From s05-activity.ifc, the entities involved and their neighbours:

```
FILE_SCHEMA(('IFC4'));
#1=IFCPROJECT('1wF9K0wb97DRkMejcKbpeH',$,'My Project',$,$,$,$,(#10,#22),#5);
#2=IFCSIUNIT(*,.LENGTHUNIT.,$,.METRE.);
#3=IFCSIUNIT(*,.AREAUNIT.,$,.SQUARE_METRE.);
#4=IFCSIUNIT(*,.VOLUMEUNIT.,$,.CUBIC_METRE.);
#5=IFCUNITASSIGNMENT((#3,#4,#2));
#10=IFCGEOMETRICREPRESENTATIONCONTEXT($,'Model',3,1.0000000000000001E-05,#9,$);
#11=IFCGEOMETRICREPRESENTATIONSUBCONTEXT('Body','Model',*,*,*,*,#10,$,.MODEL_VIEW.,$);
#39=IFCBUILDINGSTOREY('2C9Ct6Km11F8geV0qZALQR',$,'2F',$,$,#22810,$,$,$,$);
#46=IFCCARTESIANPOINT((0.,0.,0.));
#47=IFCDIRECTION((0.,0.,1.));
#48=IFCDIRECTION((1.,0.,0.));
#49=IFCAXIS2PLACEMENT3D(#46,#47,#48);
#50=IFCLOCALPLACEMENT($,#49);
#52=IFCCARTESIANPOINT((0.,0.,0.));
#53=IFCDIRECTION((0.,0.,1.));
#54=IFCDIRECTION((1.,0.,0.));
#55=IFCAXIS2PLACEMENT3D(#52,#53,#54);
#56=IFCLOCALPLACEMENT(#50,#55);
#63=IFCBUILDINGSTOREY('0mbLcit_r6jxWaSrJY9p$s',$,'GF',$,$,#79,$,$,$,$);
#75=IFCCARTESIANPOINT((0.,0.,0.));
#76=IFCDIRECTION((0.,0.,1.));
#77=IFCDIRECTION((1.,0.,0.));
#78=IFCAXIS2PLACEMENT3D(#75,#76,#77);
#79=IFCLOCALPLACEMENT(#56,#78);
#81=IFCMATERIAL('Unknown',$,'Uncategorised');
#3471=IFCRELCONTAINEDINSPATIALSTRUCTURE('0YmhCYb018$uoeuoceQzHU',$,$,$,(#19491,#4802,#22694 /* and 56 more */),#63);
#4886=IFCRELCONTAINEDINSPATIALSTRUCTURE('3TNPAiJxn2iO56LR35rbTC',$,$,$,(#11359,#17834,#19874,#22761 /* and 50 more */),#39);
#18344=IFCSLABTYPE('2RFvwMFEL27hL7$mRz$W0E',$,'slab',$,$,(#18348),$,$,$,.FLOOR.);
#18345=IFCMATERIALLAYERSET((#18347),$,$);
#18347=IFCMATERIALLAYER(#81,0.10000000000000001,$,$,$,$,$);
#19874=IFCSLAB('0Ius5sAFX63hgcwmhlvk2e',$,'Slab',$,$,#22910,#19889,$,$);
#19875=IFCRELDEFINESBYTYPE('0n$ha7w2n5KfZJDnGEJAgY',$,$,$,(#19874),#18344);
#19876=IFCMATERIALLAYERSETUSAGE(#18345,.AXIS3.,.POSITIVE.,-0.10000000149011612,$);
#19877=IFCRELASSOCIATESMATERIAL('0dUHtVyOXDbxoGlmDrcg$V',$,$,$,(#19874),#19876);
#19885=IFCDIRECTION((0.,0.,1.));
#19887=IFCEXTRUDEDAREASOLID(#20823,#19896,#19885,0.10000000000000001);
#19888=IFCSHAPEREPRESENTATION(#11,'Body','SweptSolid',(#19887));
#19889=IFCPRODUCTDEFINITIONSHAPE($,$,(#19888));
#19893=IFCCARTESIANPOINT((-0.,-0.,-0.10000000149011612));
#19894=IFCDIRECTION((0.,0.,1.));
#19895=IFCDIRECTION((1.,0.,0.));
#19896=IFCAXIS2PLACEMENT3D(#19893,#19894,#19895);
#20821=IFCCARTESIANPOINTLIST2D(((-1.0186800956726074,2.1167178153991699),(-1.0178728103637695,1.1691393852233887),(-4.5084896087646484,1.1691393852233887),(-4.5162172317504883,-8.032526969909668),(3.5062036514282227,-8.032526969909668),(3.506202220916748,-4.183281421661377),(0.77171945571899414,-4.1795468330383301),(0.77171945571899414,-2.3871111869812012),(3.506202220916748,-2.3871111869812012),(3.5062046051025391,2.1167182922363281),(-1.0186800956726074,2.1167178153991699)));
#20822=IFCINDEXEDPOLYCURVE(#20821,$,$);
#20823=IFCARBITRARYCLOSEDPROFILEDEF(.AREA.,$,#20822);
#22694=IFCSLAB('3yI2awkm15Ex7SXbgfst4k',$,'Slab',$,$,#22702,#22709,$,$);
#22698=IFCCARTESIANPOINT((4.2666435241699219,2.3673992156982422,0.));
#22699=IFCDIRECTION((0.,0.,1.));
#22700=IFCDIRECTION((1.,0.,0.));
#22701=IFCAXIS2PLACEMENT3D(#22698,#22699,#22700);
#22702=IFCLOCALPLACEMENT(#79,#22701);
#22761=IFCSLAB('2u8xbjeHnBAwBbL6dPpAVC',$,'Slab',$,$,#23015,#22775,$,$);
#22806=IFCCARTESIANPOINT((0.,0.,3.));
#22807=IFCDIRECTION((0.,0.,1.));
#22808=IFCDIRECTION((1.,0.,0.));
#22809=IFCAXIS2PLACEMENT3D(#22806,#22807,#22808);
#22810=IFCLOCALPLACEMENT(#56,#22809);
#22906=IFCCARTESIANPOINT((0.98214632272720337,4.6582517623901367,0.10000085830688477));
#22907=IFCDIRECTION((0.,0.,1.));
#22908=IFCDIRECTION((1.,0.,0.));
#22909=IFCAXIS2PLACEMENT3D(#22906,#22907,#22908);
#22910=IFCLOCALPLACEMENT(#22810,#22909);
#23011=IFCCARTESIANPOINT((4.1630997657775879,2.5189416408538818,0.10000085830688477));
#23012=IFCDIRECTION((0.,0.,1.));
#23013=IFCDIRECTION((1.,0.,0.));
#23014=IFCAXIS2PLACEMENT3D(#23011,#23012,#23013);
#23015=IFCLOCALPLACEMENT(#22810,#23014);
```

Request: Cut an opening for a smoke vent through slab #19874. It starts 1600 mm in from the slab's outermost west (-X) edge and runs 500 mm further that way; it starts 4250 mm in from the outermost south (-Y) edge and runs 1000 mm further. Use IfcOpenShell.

```python
import numpy as np
import ifcopenshell
import ifcopenshell.api.feature
import ifcopenshell.api.geometry
import ifcopenshell.api.root
import ifcopenshell.geom
import ifcopenshell.util.placement
import ifcopenshell.util.representation
import ifcopenshell.util.shape
import ifcopenshell.util.unit

model = ifcopenshell.open("s05-activity.ifc")
unit_scale = ifcopenshell.util.unit.calculate_unit_scale(model)
settings = ifcopenshell.geom.settings()


def volume(element):
    """Net volume in cubic metres, openings subtracted."""
    shape = ifcopenshell.geom.create_shape(settings, element)
    return ifcopenshell.util.shape.get_volume(shape.geometry)


slab = model.by_guid("0Ius5sAFX63hgcwmhlvk2e")
before = volume(slab)

# Extent in the slab's own axes, in metres. The edges named are its -X and -Y sides.
slab_shape = ifcopenshell.geom.create_shape(settings, slab)
vertices = ifcopenshell.util.shape.get_vertices(slab_shape.geometry)
x_min, y_min, bottom = vertices.min(axis=0)
top = vertices[:, 2].max()

opening = ifcopenshell.api.root.create_entity(model, ifc_class="IfcOpeningElement", name="Smoke vent opening", predefined_type="OPENING")
context = ifcopenshell.util.representation.get_context(model, "Model", "Body", "MODEL_VIEW")
width, depth = 0.5, 1
outline = [(0.0, 0.0), (width, 0.0), (width, depth), (0.0, depth), (0.0, 0.0)]
# Overshoot both faces by 50 mm so the cut is clean.
shape = ifcopenshell.api.geometry.add_slab_representation(
    model, context=context, depth=top - bottom + 0.1, polyline=outline
)
ifcopenshell.api.geometry.assign_representation(model, product=opening, representation=shape)

matrix = ifcopenshell.util.placement.get_local_placement(slab.ObjectPlacement)
matrix[:, 3] = matrix @ np.append(np.array([x_min + 1.6, y_min + 4.25, bottom - 0.05]) / unit_scale, 1.0)
ifcopenshell.api.geometry.edit_object_placement(model, product=opening, matrix=matrix, is_si=False)
ifcopenshell.api.feature.add_feature(model, feature=opening, element=slab)

after = volume(slab)

print(f"slab volume {before:.3f} -> {after:.3f} m3")

model.write("s05-activity_v2.ifc")
```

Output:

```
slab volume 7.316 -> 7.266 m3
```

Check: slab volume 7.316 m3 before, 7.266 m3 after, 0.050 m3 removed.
